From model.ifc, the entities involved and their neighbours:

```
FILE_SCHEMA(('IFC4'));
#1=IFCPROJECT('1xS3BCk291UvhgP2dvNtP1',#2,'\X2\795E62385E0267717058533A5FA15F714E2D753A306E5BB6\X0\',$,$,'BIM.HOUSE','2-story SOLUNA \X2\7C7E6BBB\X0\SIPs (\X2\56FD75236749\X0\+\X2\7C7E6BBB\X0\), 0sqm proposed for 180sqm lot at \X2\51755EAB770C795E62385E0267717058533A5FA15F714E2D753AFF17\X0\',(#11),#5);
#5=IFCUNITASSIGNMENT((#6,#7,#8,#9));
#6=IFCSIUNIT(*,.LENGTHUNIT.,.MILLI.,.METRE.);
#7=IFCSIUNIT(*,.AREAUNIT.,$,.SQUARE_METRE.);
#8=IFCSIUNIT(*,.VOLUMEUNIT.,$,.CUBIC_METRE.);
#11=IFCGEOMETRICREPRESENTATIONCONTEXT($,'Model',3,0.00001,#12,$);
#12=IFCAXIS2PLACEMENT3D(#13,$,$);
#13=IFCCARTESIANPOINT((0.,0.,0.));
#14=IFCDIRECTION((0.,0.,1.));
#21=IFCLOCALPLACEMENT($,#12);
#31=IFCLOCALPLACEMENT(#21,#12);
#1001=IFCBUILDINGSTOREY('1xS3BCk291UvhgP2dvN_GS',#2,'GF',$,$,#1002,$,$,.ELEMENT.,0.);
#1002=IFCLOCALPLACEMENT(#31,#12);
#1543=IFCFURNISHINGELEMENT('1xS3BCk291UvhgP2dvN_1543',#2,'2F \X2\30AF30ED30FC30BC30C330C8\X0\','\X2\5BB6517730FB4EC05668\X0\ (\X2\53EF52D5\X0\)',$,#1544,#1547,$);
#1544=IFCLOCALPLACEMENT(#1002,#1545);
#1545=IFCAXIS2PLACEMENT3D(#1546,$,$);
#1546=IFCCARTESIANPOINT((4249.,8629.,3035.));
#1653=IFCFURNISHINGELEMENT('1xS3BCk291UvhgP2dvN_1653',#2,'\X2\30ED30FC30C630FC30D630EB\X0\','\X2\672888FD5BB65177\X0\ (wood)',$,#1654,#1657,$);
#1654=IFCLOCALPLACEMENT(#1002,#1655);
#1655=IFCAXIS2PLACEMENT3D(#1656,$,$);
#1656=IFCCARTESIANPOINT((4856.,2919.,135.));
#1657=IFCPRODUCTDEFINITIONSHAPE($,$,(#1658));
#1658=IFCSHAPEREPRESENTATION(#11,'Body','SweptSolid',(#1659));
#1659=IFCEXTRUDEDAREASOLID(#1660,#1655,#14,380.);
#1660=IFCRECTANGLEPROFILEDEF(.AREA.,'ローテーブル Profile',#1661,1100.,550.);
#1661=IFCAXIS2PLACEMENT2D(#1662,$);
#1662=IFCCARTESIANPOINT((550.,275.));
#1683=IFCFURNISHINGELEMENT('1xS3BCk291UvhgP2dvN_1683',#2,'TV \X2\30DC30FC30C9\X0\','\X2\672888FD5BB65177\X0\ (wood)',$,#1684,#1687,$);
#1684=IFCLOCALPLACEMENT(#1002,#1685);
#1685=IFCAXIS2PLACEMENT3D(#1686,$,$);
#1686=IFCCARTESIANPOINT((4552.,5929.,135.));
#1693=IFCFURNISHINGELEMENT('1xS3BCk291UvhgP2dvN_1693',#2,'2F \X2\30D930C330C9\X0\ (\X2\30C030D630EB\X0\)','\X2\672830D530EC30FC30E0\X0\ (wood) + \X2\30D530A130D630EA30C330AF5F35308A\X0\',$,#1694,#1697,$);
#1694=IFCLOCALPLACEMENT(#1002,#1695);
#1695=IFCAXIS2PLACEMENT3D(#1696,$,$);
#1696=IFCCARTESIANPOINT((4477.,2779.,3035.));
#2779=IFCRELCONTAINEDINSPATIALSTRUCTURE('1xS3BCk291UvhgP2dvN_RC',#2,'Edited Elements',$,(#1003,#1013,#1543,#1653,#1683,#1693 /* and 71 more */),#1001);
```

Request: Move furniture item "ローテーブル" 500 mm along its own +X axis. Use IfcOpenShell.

```python
import ifcopenshell
import ifcopenshell.api.geometry
import ifcopenshell.util.placement
import ifcopenshell.util.unit

model = ifcopenshell.open("model.ifc")
unit_scale = ifcopenshell.util.unit.calculate_unit_scale(model)

item = model.by_guid("1xS3BCk291UvhgP2dvN_1653")
matrix = ifcopenshell.util.placement.get_local_placement(item.ObjectPlacement)
matrix[:3, 3] += matrix[:3, 0] * 0.5 / unit_scale
ifcopenshell.api.geometry.edit_object_placement(model, product=item, matrix=matrix, is_si=False)

print(ifcopenshell.util.placement.get_local_placement(item.ObjectPlacement).round(3) + 0.0)

model.write("model_edited.ifc")
```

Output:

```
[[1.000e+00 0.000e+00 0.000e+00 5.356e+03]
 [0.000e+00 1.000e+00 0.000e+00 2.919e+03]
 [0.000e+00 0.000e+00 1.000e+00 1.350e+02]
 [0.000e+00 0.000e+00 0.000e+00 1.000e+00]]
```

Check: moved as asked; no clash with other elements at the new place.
